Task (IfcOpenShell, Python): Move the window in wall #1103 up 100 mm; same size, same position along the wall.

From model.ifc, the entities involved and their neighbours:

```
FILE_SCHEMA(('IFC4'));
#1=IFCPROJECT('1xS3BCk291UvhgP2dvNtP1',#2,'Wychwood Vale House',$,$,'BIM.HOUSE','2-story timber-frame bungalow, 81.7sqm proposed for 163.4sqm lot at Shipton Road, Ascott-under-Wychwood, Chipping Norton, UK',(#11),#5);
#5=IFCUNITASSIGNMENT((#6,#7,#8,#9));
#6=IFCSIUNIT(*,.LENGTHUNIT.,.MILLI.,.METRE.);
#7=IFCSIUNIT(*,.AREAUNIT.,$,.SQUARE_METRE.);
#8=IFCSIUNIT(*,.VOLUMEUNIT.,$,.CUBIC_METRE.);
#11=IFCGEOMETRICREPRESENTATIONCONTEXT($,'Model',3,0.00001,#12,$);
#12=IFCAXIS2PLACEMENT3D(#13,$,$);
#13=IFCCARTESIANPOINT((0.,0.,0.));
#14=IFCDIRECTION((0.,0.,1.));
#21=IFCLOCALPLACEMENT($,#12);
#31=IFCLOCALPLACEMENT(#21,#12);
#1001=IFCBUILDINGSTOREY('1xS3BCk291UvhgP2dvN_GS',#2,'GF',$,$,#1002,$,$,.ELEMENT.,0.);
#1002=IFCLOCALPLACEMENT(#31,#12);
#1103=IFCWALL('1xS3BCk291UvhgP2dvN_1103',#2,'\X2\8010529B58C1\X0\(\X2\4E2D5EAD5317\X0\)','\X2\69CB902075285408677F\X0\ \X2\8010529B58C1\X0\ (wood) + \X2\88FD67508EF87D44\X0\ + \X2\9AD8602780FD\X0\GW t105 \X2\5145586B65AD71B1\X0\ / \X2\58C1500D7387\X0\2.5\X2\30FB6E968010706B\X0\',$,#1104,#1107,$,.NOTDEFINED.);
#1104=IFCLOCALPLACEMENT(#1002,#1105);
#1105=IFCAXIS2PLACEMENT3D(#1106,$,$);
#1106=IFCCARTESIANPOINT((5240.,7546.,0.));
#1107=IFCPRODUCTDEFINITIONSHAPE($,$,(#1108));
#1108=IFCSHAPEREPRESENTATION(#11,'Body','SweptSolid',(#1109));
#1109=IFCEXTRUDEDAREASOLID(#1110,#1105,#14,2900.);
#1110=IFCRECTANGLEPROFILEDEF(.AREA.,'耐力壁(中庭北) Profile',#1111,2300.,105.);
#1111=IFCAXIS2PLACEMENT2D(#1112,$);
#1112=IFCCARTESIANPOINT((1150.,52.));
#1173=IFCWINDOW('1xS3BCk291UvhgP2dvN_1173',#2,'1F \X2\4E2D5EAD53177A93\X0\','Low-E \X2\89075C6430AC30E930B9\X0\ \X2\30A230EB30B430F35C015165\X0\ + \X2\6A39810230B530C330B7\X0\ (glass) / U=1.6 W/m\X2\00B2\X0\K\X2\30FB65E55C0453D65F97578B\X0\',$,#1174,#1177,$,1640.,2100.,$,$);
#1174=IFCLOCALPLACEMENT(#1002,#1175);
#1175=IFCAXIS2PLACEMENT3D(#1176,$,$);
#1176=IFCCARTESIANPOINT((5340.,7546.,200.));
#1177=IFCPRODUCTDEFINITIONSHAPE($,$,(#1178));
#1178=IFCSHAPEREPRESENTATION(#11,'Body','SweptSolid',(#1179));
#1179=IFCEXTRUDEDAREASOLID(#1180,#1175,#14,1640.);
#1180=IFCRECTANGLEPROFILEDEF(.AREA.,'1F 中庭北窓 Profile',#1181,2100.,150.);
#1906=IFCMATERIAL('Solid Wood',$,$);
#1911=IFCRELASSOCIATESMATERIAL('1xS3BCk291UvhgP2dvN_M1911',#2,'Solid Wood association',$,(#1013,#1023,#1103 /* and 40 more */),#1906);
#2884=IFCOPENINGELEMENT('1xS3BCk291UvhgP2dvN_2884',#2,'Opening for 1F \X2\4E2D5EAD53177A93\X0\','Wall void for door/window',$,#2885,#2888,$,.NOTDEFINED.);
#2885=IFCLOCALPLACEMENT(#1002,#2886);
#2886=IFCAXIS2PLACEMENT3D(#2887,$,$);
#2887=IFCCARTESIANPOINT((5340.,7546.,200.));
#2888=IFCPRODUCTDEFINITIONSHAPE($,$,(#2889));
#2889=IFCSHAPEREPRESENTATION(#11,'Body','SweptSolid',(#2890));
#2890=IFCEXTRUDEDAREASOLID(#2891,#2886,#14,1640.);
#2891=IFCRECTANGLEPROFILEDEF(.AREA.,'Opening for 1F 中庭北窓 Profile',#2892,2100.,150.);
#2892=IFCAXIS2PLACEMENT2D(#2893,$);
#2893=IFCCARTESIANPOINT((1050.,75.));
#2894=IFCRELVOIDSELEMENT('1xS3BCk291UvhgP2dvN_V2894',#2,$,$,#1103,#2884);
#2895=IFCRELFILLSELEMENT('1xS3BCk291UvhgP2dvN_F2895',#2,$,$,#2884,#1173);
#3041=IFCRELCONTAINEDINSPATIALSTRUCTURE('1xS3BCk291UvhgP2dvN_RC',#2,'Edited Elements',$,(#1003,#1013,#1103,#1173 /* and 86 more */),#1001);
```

```python
import numpy as np
import ifcopenshell
import ifcopenshell.api.geometry
import ifcopenshell.util.placement
import ifcopenshell.util.unit

model = ifcopenshell.open("model.ifc")
unit_scale = ifcopenshell.util.unit.calculate_unit_scale(model)

window = model.by_guid("1xS3BCk291UvhgP2dvN_1173")
opening = window.FillsVoids[0].RelatingOpeningElement
dz = 0.1 / unit_scale

shift = np.array([0.0, 0.0, dz])
# The window is not placed relative to its opening, so move both.
for product in (opening, window):
    matrix = ifcopenshell.util.placement.get_local_placement(product.ObjectPlacement)
    matrix[:3, 3] += shift
    ifcopenshell.api.geometry.edit_object_placement(model, product=product, matrix=matrix, is_si=False)

print(f"moved by {dz * unit_scale:+.3f} m")

model.write("model_edited.ifc")
```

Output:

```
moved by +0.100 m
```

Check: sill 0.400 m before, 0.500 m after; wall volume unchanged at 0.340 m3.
